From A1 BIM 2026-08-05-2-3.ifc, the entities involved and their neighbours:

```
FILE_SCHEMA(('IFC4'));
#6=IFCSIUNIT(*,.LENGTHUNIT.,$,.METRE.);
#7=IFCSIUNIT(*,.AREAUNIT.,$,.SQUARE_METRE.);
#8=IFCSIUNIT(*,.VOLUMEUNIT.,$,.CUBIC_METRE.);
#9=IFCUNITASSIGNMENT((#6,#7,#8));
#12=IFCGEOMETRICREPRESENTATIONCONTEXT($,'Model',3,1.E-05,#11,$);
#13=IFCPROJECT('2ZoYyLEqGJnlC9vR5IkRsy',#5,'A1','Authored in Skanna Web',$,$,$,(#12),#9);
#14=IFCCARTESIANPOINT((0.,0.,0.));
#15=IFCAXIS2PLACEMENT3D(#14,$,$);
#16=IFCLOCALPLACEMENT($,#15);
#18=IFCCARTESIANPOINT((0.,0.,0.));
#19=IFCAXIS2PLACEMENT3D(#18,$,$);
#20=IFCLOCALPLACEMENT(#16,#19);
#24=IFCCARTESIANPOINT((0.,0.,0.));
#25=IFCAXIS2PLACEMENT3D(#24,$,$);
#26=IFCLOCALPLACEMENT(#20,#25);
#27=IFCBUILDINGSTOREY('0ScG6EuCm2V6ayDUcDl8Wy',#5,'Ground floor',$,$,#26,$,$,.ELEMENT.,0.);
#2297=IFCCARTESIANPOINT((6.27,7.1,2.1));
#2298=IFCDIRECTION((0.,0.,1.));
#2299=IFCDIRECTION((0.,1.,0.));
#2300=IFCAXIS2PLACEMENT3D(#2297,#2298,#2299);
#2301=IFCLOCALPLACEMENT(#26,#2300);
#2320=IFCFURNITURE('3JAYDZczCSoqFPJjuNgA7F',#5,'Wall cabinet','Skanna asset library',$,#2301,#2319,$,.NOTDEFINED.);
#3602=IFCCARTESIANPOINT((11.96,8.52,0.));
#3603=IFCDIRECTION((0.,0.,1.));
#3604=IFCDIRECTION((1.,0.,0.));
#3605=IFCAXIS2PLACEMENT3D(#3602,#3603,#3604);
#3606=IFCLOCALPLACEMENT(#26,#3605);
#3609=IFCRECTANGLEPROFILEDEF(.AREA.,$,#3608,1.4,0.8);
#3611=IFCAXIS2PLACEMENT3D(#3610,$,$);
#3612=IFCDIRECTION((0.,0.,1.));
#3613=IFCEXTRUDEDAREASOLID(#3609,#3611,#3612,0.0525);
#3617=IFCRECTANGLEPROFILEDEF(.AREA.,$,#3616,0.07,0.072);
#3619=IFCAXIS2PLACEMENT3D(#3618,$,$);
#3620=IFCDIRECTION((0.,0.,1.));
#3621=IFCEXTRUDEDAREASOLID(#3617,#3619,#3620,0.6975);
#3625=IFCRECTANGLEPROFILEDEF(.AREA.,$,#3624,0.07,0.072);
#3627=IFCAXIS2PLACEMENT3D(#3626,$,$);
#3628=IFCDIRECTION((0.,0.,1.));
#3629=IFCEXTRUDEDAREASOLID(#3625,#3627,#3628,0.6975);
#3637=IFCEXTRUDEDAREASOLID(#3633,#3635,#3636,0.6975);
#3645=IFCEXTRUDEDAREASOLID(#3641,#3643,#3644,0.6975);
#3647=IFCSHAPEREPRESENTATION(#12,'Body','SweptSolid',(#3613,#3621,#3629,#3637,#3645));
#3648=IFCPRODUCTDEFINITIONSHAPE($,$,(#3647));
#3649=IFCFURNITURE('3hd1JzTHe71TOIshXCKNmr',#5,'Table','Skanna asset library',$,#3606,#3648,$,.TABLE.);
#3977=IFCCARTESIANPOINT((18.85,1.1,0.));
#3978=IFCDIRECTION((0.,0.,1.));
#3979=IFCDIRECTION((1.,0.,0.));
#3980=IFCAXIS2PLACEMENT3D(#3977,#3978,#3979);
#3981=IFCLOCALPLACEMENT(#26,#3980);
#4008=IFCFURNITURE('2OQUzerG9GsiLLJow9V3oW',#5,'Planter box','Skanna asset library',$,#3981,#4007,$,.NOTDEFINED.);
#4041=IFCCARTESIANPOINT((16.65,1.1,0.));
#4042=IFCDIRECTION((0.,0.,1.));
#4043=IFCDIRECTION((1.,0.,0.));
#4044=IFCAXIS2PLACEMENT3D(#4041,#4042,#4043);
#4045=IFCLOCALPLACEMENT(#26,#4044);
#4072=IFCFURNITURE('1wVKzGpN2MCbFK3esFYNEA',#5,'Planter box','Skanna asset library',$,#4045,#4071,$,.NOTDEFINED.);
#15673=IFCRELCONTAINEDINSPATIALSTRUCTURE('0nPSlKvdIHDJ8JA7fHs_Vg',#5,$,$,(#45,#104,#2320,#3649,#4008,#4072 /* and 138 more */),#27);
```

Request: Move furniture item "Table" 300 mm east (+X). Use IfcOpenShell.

```python
import ifcopenshell
import ifcopenshell.api.geometry
import ifcopenshell.util.placement
import ifcopenshell.util.unit

model = ifcopenshell.open("A1 BIM 2026-08-05-2-3.ifc")
unit_scale = ifcopenshell.util.unit.calculate_unit_scale(model)

item = model.by_id(3649)
matrix = ifcopenshell.util.placement.get_local_placement(item.ObjectPlacement)
matrix[0, 3] += 0.3 / unit_scale
ifcopenshell.api.geometry.edit_object_placement(model, product=item, matrix=matrix, is_si=False)

print(ifcopenshell.util.placement.get_local_placement(item.ObjectPlacement).round(3) + 0.0)

model.write("A1 BIM 2026-08-05-2-3_rev.ifc")
```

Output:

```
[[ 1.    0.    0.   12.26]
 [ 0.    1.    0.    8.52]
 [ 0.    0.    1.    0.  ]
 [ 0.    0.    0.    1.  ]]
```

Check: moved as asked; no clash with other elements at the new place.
